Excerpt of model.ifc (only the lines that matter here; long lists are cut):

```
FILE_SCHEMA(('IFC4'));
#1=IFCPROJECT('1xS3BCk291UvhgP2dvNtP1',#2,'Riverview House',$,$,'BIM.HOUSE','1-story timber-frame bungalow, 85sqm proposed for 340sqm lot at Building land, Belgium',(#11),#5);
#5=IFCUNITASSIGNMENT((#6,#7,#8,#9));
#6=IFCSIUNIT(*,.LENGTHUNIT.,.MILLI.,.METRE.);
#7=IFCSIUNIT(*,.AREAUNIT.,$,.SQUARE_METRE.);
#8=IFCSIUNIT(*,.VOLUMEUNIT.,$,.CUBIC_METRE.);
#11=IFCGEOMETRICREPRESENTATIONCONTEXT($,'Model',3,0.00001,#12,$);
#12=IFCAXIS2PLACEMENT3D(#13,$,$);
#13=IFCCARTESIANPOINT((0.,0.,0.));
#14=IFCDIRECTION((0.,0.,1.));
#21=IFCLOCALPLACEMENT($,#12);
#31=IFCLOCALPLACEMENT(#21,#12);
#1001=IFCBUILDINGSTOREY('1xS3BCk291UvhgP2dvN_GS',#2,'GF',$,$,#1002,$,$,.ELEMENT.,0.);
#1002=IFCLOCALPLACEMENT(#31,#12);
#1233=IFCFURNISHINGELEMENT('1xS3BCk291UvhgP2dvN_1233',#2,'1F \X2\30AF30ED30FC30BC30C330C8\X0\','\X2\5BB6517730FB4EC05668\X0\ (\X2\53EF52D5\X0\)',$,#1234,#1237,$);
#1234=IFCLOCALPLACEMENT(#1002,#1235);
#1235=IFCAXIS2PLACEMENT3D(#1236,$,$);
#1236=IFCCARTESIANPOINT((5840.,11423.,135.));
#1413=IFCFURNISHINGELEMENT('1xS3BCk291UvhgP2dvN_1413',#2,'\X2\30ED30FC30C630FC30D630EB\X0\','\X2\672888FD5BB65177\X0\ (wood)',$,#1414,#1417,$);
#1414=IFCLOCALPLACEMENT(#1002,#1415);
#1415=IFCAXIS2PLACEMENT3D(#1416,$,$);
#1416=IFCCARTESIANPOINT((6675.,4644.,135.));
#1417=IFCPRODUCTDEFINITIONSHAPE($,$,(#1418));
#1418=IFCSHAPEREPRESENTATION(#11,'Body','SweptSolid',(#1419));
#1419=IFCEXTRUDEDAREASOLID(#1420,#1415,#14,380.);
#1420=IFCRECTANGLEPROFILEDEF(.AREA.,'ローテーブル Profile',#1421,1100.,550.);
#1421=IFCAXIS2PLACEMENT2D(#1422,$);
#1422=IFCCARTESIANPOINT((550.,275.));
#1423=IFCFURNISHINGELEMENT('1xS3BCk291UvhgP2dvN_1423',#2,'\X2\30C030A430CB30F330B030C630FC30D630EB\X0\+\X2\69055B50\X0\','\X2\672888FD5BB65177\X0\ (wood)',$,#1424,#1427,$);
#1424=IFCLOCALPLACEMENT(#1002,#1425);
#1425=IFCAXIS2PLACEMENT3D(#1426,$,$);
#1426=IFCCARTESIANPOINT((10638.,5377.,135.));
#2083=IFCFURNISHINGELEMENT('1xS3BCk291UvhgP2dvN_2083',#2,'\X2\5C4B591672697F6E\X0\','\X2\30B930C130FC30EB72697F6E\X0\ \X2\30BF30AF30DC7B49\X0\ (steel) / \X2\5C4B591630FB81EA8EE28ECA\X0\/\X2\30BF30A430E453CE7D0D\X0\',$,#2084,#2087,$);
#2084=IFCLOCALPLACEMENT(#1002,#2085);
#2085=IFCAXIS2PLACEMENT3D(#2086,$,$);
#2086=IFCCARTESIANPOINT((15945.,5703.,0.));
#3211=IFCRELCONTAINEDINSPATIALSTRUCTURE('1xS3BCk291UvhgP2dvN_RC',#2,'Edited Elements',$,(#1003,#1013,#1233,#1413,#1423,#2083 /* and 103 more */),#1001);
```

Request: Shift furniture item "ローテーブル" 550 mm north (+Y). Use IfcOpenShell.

```python
import ifcopenshell
import ifcopenshell.api.geometry
import ifcopenshell.util.placement

model = ifcopenshell.open("model.ifc")

item = model.by_guid("1xS3BCk291UvhgP2dvN_1413")
matrix = ifcopenshell.util.placement.get_local_placement(item.ObjectPlacement)
matrix[1, 3] += 550.0
ifcopenshell.api.geometry.edit_object_placement(model, product=item, matrix=matrix, is_si=False)

print(ifcopenshell.util.placement.get_local_placement(item.ObjectPlacement).round(3) + 0.0)

model.write("model_v2.ifc")
```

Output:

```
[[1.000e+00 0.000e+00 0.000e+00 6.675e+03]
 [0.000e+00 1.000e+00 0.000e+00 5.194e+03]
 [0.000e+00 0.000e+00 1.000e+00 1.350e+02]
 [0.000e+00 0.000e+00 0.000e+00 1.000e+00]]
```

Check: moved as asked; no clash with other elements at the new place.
